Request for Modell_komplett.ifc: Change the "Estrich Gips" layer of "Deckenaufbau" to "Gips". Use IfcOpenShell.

First a look at what the model holds.

```python
import ifcopenshell
import ifcopenshell.util.element

model = ifcopenshell.open("Modell_komplett.ifc")
print(model.schema)
for layer_set in model.by_type("IfcMaterialLayerSet"):
    if layer_set.LayerSetName == "Deckenaufbau":
        for layer in layer_set.MaterialLayers:
            print(layer.id(), layer.Material and layer.Material.Name, layer.LayerThickness, sep=" | ")
        print(len(ifcopenshell.util.element.get_elements_by_material(model, layer_set)), "elements and types use it")
print(sorted(m.Name for m in model.by_type("IfcMaterial") if m.Name)[:60])
```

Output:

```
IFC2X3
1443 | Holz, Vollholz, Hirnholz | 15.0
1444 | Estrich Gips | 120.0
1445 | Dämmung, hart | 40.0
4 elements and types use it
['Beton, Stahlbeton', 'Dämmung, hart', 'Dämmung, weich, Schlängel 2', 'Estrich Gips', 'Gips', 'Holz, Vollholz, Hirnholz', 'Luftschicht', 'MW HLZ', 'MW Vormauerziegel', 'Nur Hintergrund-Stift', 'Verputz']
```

```python
import ifcopenshell
import ifcopenshell.api.material

model = ifcopenshell.open("Modell_komplett.ifc")

layer_set = next(s for s in model.by_type("IfcMaterialLayerSet") if s.LayerSetName == "Deckenaufbau")
layer = next(l for l in layer_set.MaterialLayers if l.Material and l.Material.Name == "Estrich Gips")
material = next(m for m in model.by_type("IfcMaterial") if m.Name == "Gips")

# Point this one layer at the other material; renaming the old one would change it everywhere.
ifcopenshell.api.material.edit_layer(model, layer=layer, attributes={}, material=material)

print([l.Material.Name if l.Material else None for l in layer_set.MaterialLayers])

model.write("Modell_komplett_edited.ifc")
```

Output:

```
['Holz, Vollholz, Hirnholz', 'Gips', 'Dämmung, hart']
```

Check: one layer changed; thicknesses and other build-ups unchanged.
